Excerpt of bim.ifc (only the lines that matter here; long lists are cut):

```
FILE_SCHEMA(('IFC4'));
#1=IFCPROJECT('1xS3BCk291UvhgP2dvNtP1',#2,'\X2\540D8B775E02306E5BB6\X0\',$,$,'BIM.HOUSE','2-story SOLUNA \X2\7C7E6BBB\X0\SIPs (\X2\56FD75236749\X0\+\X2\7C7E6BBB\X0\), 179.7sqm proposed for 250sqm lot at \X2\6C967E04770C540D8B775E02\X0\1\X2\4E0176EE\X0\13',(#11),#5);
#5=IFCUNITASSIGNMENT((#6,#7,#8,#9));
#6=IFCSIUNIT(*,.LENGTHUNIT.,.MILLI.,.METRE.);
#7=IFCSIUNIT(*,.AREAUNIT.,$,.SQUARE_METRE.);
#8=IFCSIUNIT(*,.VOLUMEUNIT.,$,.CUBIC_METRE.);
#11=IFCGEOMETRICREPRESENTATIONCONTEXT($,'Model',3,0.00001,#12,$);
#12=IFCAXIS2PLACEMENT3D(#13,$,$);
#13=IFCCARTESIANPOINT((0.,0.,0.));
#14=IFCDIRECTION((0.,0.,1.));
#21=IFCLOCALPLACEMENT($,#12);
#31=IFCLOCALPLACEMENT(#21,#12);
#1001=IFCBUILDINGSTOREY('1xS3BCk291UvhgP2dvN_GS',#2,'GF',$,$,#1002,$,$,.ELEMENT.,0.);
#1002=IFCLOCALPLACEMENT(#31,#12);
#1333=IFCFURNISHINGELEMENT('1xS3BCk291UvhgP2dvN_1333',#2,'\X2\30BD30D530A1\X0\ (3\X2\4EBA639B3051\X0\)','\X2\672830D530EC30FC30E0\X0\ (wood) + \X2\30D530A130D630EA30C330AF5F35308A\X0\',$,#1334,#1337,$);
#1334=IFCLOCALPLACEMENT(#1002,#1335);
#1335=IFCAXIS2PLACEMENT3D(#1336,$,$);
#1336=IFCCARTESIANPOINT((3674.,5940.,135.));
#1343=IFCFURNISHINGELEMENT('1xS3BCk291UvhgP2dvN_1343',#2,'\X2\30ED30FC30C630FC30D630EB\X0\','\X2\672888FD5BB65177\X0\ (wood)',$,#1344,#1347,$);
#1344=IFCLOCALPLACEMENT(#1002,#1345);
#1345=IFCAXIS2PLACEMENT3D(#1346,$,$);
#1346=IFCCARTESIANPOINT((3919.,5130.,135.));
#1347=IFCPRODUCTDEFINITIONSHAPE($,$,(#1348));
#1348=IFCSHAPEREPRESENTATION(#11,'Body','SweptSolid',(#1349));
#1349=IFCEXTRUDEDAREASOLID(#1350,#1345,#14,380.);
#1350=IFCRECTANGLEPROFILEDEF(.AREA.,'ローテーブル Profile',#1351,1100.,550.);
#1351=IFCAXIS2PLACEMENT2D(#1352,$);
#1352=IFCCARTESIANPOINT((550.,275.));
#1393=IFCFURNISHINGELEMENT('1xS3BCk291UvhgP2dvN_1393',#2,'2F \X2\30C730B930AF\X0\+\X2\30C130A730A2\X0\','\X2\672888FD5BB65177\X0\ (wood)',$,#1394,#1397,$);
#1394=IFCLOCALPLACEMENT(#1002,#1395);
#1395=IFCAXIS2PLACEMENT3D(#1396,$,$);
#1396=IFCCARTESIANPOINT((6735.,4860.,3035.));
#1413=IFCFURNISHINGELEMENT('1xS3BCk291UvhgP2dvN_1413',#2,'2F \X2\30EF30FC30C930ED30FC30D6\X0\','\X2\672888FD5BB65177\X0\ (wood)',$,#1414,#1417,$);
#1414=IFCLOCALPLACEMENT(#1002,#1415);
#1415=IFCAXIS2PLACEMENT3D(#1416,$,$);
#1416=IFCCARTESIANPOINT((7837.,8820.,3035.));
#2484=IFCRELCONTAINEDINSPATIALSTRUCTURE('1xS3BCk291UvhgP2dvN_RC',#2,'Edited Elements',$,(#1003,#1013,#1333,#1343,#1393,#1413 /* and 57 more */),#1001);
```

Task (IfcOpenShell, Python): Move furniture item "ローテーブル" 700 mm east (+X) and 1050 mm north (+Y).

```python
import ifcopenshell
import ifcopenshell.api.geometry
import ifcopenshell.util.placement

model = ifcopenshell.open("bim.ifc")

item = model.by_id(1343)
matrix = ifcopenshell.util.placement.get_local_placement(item.ObjectPlacement)
matrix[0, 3] += 700.0
matrix[1, 3] += 1050.0
ifcopenshell.api.geometry.edit_object_placement(model, product=item, matrix=matrix, is_si=False)

print(ifcopenshell.util.placement.get_local_placement(item.ObjectPlacement).round(3) + 0.0)

model.write("bim-out.ifc")
```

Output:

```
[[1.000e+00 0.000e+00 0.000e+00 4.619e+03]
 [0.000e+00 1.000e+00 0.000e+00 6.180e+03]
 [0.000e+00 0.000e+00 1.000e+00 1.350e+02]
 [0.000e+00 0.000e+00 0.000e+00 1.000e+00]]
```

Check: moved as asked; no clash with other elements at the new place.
